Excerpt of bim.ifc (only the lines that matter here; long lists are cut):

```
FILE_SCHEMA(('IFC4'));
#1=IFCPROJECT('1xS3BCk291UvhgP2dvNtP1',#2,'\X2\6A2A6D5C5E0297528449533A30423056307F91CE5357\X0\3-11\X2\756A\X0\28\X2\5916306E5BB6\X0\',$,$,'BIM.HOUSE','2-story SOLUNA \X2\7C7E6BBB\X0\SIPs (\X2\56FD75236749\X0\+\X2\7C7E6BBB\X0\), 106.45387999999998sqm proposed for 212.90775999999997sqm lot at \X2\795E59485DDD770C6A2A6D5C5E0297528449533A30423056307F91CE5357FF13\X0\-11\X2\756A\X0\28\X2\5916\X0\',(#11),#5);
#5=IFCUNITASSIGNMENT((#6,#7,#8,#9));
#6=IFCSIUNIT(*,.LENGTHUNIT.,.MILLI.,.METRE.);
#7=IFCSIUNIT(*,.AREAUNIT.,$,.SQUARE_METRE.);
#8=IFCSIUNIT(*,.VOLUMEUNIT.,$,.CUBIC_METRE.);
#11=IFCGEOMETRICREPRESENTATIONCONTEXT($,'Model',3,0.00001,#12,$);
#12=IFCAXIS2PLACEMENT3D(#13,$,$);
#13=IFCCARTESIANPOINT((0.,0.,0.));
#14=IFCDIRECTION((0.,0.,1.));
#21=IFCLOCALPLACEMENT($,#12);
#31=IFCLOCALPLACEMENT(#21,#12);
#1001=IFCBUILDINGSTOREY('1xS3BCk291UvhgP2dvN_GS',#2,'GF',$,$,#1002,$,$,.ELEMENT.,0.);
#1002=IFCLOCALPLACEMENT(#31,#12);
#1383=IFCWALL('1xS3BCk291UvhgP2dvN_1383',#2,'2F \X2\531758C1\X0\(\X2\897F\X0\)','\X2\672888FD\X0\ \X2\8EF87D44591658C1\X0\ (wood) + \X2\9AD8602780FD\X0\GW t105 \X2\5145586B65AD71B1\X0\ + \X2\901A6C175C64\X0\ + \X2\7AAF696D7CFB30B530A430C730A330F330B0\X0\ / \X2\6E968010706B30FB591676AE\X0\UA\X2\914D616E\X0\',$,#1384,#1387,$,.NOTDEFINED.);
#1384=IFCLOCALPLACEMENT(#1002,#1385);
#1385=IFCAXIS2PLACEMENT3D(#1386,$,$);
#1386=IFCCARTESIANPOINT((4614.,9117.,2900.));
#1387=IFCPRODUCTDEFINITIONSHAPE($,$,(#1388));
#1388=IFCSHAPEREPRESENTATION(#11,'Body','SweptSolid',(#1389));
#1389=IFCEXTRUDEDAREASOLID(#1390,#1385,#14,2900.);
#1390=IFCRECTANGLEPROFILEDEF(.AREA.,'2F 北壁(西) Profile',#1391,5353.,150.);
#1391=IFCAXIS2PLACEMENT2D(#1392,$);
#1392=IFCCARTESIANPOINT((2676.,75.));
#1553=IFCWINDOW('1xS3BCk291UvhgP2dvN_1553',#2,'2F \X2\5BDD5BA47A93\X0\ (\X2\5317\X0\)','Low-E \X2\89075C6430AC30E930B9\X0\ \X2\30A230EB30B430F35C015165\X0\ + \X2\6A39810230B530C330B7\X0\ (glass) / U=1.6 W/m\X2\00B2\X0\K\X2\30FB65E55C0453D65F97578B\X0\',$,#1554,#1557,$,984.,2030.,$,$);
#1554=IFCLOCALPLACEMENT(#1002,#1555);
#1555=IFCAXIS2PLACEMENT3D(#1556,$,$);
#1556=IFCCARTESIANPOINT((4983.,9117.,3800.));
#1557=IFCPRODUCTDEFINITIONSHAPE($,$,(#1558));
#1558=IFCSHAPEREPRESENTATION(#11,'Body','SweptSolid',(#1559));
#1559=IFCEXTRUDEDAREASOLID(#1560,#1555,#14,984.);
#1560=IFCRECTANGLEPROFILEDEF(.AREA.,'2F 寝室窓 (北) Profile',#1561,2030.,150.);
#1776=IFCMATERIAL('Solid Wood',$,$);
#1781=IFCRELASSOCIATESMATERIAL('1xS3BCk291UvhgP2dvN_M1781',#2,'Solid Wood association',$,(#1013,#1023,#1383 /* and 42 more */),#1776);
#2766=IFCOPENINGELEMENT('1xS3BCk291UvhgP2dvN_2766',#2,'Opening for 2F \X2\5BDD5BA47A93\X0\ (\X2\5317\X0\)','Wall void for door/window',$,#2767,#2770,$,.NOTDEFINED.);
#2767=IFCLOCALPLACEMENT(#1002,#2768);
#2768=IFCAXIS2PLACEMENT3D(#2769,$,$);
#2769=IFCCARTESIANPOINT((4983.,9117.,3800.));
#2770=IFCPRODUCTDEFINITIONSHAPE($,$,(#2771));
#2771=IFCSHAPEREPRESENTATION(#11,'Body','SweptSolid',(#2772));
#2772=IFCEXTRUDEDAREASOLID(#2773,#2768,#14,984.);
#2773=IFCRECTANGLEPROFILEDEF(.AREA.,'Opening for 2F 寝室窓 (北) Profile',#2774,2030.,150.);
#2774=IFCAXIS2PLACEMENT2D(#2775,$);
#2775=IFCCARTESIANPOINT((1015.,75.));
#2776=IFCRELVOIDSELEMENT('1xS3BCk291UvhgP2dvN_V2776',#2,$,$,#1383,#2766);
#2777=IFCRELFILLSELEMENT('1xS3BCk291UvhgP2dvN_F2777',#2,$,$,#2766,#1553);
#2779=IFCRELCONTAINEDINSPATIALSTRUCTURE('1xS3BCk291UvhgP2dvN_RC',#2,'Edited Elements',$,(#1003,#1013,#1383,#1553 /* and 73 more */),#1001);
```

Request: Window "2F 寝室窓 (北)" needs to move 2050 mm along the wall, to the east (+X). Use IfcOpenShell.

```python
import ifcopenshell
import ifcopenshell.api.geometry
import ifcopenshell.util.placement

model = ifcopenshell.open("bim.ifc")

window = model.by_guid("1xS3BCk291UvhgP2dvN_1553")
opening = window.FillsVoids[0].RelatingOpeningElement
wall = opening.VoidsElements[0].RelatingBuildingElement

wall_matrix = ifcopenshell.util.placement.get_local_placement(wall.ObjectPlacement)
shift = wall_matrix[:3, 0] * 2050.0
before = ifcopenshell.util.placement.get_local_placement(window.ObjectPlacement)[:3, 3].copy()

# The window is not placed relative to its opening, so move both.
for product in (opening, window):
    matrix = ifcopenshell.util.placement.get_local_placement(product.ObjectPlacement)
    matrix[:3, 3] += shift
    ifcopenshell.api.geometry.edit_object_placement(model, product=product, matrix=matrix, is_si=False)

after = ifcopenshell.util.placement.get_local_placement(window.ObjectPlacement)[:3, 3]
print("window moved by", (after - before).round(3) + 0.0)

model.write("bim_edited.ifc")
```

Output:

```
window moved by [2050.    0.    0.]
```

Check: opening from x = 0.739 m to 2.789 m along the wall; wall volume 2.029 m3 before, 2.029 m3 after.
